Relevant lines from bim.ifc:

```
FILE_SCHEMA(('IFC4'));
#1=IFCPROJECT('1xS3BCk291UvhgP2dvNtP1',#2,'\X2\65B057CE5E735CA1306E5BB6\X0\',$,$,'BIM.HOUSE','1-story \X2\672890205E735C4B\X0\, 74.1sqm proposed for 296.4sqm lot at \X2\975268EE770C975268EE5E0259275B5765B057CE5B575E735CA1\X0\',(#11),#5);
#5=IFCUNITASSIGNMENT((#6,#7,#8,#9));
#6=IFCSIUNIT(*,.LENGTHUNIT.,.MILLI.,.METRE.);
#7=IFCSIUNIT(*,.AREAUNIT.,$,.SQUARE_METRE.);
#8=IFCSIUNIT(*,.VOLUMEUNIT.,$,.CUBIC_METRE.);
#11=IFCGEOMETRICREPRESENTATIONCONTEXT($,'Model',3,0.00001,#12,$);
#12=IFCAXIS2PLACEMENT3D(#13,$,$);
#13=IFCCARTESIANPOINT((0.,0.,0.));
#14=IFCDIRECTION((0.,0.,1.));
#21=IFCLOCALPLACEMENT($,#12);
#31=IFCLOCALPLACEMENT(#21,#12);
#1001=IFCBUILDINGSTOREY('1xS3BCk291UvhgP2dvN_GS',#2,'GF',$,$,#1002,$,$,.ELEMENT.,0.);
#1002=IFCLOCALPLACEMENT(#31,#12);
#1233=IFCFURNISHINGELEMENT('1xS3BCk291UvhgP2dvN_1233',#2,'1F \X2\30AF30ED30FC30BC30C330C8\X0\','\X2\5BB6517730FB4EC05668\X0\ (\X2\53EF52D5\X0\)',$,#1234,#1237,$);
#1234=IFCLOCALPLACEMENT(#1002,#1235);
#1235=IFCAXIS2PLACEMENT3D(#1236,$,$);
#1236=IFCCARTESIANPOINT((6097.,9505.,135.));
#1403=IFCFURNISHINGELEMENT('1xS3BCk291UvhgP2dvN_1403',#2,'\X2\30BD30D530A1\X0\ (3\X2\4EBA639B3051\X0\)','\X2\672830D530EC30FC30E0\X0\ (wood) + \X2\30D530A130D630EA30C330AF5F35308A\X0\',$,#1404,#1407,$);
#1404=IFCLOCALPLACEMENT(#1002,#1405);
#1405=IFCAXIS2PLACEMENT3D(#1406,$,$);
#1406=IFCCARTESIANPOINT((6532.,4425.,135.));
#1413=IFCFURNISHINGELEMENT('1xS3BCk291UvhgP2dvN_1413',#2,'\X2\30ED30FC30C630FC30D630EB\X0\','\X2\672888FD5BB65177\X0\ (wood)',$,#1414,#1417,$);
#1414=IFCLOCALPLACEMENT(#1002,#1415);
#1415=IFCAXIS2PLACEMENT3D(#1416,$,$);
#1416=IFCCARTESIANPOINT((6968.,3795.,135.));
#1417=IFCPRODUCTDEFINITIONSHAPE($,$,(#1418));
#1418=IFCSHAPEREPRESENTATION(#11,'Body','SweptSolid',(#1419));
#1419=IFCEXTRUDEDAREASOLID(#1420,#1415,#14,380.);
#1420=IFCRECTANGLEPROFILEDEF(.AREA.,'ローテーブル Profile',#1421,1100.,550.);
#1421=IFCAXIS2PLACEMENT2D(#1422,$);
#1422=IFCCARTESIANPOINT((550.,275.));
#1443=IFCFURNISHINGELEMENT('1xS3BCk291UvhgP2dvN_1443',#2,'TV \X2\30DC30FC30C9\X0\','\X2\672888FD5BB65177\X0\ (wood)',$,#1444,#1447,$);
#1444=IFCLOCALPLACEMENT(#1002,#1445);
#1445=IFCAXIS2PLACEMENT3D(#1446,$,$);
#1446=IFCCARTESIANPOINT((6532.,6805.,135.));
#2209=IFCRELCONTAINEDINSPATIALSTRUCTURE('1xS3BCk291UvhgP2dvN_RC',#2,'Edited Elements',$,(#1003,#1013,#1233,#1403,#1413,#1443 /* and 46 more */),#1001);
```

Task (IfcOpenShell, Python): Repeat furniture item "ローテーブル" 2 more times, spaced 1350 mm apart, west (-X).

```python
import numpy as np
import ifcopenshell
import ifcopenshell.api.geometry
import ifcopenshell.api.root
import ifcopenshell.util.element
import ifcopenshell.util.placement
import ifcopenshell.util.unit

model = ifcopenshell.open("bim.ifc")
unit_scale = ifcopenshell.util.unit.calculate_unit_scale(model)


def reuse_history(source, copy):
    """copy_class also copies each property set's owner history, people and application; keep the originals."""
    for rel in copy.IsDefinedBy:
        if rel.is_a("IfcRelDefinesByProperties") and (history := rel.RelatingPropertyDefinition.OwnerHistory):
            rel.RelatingPropertyDefinition.OwnerHistory = source.OwnerHistory
            ifcopenshell.util.element.remove_deep2(model, history)


source = model.by_guid("1xS3BCk291UvhgP2dvN_1413")
base = ifcopenshell.util.placement.get_local_placement(source.ObjectPlacement)
step = np.array([-1.0, 0.0, 0.0]) * 1.35 / unit_scale

for i in range(1, 3):
    copy = ifcopenshell.api.root.copy_class(model, product=source)
    copy.Representation = ifcopenshell.util.element.copy_deep(
        model, source.Representation, exclude=["IfcGeometricRepresentationContext", "IfcRepresentationMap"]
    )
    reuse_history(source, copy)
    matrix = base.copy()
    matrix[:3, 3] += i * step
    print("added at", matrix[:3, 3].round(3) + 0.0)
    ifcopenshell.api.geometry.edit_object_placement(model, product=copy, matrix=matrix, is_si=False)

model.write("bim_rev.ifc")
```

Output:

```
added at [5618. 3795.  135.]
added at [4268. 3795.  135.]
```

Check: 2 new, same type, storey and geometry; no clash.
